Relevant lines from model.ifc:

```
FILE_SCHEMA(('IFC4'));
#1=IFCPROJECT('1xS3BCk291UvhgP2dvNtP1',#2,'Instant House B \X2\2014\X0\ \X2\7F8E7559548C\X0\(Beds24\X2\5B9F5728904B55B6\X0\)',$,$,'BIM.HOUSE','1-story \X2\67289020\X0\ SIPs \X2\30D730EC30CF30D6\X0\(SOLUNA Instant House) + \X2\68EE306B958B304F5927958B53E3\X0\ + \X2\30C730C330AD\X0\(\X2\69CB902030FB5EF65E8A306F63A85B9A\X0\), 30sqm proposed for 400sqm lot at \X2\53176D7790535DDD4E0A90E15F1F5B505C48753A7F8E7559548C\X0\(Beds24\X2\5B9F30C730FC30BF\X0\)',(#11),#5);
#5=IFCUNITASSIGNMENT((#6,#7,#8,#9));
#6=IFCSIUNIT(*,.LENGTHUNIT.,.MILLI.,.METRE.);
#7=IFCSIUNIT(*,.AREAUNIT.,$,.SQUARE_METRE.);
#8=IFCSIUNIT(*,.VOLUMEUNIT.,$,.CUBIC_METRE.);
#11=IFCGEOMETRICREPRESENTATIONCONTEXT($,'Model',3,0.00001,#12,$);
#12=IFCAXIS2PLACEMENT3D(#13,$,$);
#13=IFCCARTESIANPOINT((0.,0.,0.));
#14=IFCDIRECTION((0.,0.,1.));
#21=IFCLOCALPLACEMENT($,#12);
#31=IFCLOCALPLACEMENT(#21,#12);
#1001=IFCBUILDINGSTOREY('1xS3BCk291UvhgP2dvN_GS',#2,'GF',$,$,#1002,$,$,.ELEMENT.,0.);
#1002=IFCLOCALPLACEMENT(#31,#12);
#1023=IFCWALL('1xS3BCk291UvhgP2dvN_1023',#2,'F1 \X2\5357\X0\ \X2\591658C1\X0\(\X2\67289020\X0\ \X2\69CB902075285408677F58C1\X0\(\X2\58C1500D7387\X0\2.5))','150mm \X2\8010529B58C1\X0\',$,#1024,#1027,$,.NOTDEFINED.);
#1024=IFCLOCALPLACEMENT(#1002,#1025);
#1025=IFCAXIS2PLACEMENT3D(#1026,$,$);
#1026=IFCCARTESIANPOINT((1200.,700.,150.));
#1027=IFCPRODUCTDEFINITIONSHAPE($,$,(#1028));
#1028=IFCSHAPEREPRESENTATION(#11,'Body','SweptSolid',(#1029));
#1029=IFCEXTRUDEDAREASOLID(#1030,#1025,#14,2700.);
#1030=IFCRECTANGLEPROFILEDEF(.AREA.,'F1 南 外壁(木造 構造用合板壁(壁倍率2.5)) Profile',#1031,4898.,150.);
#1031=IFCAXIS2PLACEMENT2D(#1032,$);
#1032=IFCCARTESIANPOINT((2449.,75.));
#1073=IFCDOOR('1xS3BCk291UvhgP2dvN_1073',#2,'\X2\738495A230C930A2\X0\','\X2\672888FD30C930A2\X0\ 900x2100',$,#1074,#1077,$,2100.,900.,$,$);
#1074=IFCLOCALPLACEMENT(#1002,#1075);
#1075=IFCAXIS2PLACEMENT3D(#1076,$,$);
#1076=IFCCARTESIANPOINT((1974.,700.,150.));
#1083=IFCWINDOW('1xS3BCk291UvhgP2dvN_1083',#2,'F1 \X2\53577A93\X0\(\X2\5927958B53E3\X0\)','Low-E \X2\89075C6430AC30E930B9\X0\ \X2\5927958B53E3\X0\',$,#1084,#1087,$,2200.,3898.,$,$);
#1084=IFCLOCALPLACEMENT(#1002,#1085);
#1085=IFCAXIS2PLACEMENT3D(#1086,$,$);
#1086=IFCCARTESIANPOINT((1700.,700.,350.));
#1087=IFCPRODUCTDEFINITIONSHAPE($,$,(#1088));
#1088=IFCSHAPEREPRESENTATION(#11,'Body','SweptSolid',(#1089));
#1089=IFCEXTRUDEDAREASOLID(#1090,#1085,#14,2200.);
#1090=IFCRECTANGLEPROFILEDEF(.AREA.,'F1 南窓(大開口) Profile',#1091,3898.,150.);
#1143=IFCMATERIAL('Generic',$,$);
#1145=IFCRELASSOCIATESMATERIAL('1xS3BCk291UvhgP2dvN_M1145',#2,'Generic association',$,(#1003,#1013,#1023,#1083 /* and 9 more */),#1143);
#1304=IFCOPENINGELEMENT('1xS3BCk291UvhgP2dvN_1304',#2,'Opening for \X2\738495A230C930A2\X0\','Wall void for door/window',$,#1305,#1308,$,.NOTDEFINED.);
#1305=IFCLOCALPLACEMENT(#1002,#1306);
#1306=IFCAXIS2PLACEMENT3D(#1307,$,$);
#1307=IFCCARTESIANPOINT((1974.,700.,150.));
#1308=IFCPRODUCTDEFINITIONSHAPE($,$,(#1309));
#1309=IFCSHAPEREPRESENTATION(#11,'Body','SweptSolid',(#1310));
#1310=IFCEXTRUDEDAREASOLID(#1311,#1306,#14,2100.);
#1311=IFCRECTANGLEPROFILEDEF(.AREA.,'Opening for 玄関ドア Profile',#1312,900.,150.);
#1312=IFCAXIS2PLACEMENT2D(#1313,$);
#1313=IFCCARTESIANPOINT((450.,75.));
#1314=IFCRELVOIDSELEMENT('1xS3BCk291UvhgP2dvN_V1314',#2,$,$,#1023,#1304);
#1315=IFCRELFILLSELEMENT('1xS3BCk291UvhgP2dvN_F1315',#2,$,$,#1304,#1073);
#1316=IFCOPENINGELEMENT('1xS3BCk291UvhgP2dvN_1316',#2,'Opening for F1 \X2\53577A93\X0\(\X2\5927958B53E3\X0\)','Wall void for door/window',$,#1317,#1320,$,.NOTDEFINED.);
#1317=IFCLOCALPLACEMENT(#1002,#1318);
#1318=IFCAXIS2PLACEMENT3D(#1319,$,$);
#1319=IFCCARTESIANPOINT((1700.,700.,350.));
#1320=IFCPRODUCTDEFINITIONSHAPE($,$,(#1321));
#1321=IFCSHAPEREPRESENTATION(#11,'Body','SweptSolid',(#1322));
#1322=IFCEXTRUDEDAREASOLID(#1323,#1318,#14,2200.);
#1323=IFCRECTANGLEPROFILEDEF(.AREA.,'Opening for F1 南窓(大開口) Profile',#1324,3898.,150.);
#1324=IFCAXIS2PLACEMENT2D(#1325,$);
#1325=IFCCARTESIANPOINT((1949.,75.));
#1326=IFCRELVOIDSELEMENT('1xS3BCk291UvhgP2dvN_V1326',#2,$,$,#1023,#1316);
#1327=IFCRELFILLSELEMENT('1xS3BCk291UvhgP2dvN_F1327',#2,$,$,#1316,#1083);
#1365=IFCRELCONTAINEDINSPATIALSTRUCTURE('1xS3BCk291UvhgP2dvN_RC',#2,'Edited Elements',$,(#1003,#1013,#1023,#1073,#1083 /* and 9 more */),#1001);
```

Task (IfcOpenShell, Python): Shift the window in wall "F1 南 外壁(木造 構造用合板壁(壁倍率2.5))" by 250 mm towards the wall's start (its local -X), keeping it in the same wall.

```python
import ifcopenshell
import ifcopenshell.api.geometry
import ifcopenshell.util.placement

model = ifcopenshell.open("model.ifc")

window = model.by_guid("1xS3BCk291UvhgP2dvN_1083")
opening = window.FillsVoids[0].RelatingOpeningElement
wall = opening.VoidsElements[0].RelatingBuildingElement

wall_matrix = ifcopenshell.util.placement.get_local_placement(wall.ObjectPlacement)
shift = wall_matrix[:3, 0] * -250.0
before = ifcopenshell.util.placement.get_local_placement(window.ObjectPlacement)[:3, 3].copy()

# The window is not placed relative to its opening, so move both.
for product in (opening, window):
    matrix = ifcopenshell.util.placement.get_local_placement(product.ObjectPlacement)
    matrix[:3, 3] += shift
    ifcopenshell.api.geometry.edit_object_placement(model, product=product, matrix=matrix, is_si=False)

after = ifcopenshell.util.placement.get_local_placement(window.ObjectPlacement)[:3, 3]
print("window moved by", (after - before).round(3) + 0.0)

model.write("model_v2.ifc")
```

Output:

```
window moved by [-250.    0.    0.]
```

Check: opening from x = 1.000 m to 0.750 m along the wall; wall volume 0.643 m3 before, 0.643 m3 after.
